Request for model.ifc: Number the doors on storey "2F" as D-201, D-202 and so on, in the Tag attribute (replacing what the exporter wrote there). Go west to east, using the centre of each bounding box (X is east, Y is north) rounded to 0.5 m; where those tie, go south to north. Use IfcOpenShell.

First a look at what the model holds.

```python
import ifcopenshell
import ifcopenshell.util.element
import ifcopenshell.util.placement

model = ifcopenshell.open("model.ifc")
print(model.schema)
storey = next(s for s in model.by_type("IfcBuildingStorey") if s.Name == "2F")
doors = [e for e in ifcopenshell.util.element.get_decomposition(storey) if e.is_a("IfcDoor")]
for e in sorted(doors, key=lambda e: e.id()):
    origin = ifcopenshell.util.placement.get_local_placement(e.ObjectPlacement)[:3, 3]
    print(e.id(), e.Tag, e.Name, origin.round(2) + 0.0, sep=" | ")
```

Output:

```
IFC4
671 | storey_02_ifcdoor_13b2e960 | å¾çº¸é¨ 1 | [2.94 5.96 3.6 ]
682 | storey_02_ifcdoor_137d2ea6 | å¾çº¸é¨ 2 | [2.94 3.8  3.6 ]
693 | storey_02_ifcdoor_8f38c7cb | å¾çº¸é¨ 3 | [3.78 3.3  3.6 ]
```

```python
import ifcopenshell
import ifcopenshell.geom
import ifcopenshell.util.element
import ifcopenshell.util.shape

model = ifcopenshell.open("model.ifc")
settings = ifcopenshell.geom.settings()
settings.set("use-world-coords", True)


def centre(element):
    shape = ifcopenshell.geom.create_shape(settings, element)
    return ifcopenshell.util.shape.get_bbox_centroid(shape.geometry)


storey = next(s for s in model.by_type("IfcBuildingStorey") if s.Name == "2F")
doors = [e for e in ifcopenshell.util.element.get_decomposition(storey) if e.is_a("IfcDoor")]

# Insertion points can sit at a corner or the storey origin, so sort by the geometry (in metres).
centres = {e: centre(e) for e in doors}
doors.sort(key=lambda e: (round(centres[e][0] / 0.5), centres[e][1]))

for i, e in enumerate(doors, start=1):
    number = f"D-2{i:02d}"
    e.Tag = number
    print(e.id(), number)

model.write("model_updated.ifc")
```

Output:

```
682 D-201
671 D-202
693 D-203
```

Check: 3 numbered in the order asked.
